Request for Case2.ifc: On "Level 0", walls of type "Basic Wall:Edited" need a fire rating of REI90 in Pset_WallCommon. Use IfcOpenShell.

First a look at what the model holds.

```python
import ifcopenshell
import ifcopenshell.util.element

model = ifcopenshell.open("Case2.ifc")
print(model.schema)
storey = next(s for s in model.by_type("IfcBuildingStorey") if s.Name == "Level 0")
walls = [e for e in ifcopenshell.util.element.get_decomposition(storey) if e.is_a("IfcWall")]
seen = {}
for e in walls:
    element_type = ifcopenshell.util.element.get_type(e)
    key = (element_type.Name if element_type != e and element_type else None, ifcopenshell.util.element.get_pset(e, "Pset_WallCommon", "FireRating"))
    seen[key] = seen.get(key, 0) + 1
for (name, value), count in sorted(seen.items(), key=str):
    print(count, "x", name, "|", value)
```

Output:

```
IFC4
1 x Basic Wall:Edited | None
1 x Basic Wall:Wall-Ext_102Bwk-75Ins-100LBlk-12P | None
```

```python
import ifcopenshell
import ifcopenshell.api.pset
import ifcopenshell.util.element

model = ifcopenshell.open("Case2.ifc")

storey = next(s for s in model.by_type("IfcBuildingStorey") if s.Name == "Level 0")
walls = [e for e in ifcopenshell.util.element.get_decomposition(storey) if e.is_a("IfcWall")]

count = 0
for e in walls:
    element_type = ifcopenshell.util.element.get_type(e)
    if element_type in (None, e) or element_type.Name != "Basic Wall:Edited":
        continue
    # add_pset returns the element's existing set when there is one.
    pset = ifcopenshell.api.pset.add_pset(model, product=e, name="Pset_WallCommon")
    ifcopenshell.api.pset.edit_pset(model, pset=pset, properties={"FireRating": "REI90"})
    count += 1

print(count, "walls updated")

model.write("Case2_updated.ifc")
```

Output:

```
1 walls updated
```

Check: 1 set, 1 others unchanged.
